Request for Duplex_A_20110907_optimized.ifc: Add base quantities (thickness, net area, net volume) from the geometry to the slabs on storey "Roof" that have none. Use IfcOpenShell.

First a look at what the model holds.

```python
import ifcopenshell
import ifcopenshell.util.element
import ifcopenshell.util.unit

model = ifcopenshell.open("Duplex_A_20110907_optimized.ifc")
print(model.schema)
for unit_type in ("LENGTHUNIT", "AREAUNIT", "VOLUMEUNIT"):
    print(unit_type, ifcopenshell.util.unit.calculate_unit_scale(model, unit_type))
storey = next(s for s in model.by_type("IfcBuildingStorey") if s.Name == "Roof")
slabs = [e for e in ifcopenshell.util.element.get_decomposition(storey) if e.is_a("IfcSlab")]
for e in sorted(slabs, key=lambda e: e.id()):
    print(e.id(), e.is_a(), e.Name, list(ifcopenshell.util.element.get_psets(e, qtos_only=True)), sep=" | ")
```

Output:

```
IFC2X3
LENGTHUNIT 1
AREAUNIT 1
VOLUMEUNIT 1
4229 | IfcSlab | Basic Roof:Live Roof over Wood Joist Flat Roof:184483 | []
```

```python
import ifcopenshell
import ifcopenshell.api.pset
import ifcopenshell.geom
import ifcopenshell.util.element
import ifcopenshell.util.shape
import ifcopenshell.util.unit

model = ifcopenshell.open("Duplex_A_20110907_optimized.ifc")
unit_scale = ifcopenshell.util.unit.calculate_unit_scale(model)
area_scale = ifcopenshell.util.unit.calculate_unit_scale(model, "AREAUNIT")
volume_scale = ifcopenshell.util.unit.calculate_unit_scale(model, "VOLUMEUNIT")
settings = ifcopenshell.geom.settings()

storey = next(s for s in model.by_type("IfcBuildingStorey") if s.Name == "Roof")
slabs = [e for e in ifcopenshell.util.element.get_decomposition(storey) if e.is_a("IfcSlab")]

for e in sorted(slabs, key=lambda e: e.id()):
    if ifcopenshell.util.element.get_psets(e, qtos_only=True, should_inherit=False):
        continue
    # Geometry comes back in metres, in the element's own axes.
    shape = ifcopenshell.geom.create_shape(settings, e)
    values = {
        "Width": ifcopenshell.util.shape.get_z(shape.geometry) / unit_scale,
        "NetArea": ifcopenshell.util.shape.get_footprint_area(shape.geometry) / area_scale,
        "NetVolume": ifcopenshell.util.shape.get_volume(shape.geometry) / volume_scale,
    }
    qto = ifcopenshell.api.pset.add_qto(model, product=e, name="BaseQuantities")
    ifcopenshell.api.pset.edit_qto(model, qto=qto, properties=values)
    print(e.id(), {k: round(v, 3) for k, v in values.items()})

model.write("Duplex_A_20110907_optimized_rev.ifc")
```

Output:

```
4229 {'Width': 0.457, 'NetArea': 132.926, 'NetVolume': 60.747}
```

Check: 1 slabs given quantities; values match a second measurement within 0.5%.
